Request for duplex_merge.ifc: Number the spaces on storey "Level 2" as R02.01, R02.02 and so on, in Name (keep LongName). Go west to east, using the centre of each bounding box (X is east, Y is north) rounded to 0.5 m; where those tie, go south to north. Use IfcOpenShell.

First a look at what the model holds.

```python
import ifcopenshell
import ifcopenshell.util.element
import ifcopenshell.util.placement

model = ifcopenshell.open("duplex_merge.ifc")
print(model.schema)
storey = next(s for s in model.by_type("IfcBuildingStorey") if s.Name == "Level 2")
spaces = [e for e in ifcopenshell.util.element.get_decomposition(storey) if e.is_a("IfcSpace")]
for e in sorted(spaces, key=lambda e: e.id()):
    origin = ifcopenshell.util.placement.get_local_placement(e.ObjectPlacement)[:3, 3]
    print(e.id(), e.Name, e.LongName, origin.round(2) + 0.0, sep=" | ")
```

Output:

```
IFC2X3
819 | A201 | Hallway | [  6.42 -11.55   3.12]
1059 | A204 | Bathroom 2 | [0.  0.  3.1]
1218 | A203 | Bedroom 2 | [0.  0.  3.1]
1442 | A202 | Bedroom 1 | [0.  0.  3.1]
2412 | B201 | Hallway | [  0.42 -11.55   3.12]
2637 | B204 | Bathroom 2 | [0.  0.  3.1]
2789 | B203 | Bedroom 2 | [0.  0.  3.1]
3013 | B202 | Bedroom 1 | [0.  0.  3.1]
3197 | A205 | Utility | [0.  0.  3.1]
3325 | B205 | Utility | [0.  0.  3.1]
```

```python
import ifcopenshell
import ifcopenshell.geom
import ifcopenshell.util.element
import ifcopenshell.util.shape

model = ifcopenshell.open("duplex_merge.ifc")
settings = ifcopenshell.geom.settings()
settings.set("use-world-coords", True)


def centre(element):
    shape = ifcopenshell.geom.create_shape(settings, element)
    return ifcopenshell.util.shape.get_bbox_centroid(shape.geometry)


storey = next(s for s in model.by_type("IfcBuildingStorey") if s.Name == "Level 2")
spaces = [e for e in ifcopenshell.util.element.get_decomposition(storey) if e.is_a("IfcSpace")]

# Insertion points can sit at a corner or the storey origin, so sort by the geometry (in metres).
centres = {e: centre(e) for e in spaces}
spaces.sort(key=lambda e: (round(centres[e][0] / 0.5), centres[e][1]))

for i, e in enumerate(spaces, start=1):
    number = f"R02.{i:02d}"
    e.Name = number
    print(e.id(), number)

model.write("duplex_merge_rev.ifc")
```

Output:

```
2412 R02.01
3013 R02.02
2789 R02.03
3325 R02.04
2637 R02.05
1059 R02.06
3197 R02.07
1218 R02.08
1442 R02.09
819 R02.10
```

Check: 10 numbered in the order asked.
